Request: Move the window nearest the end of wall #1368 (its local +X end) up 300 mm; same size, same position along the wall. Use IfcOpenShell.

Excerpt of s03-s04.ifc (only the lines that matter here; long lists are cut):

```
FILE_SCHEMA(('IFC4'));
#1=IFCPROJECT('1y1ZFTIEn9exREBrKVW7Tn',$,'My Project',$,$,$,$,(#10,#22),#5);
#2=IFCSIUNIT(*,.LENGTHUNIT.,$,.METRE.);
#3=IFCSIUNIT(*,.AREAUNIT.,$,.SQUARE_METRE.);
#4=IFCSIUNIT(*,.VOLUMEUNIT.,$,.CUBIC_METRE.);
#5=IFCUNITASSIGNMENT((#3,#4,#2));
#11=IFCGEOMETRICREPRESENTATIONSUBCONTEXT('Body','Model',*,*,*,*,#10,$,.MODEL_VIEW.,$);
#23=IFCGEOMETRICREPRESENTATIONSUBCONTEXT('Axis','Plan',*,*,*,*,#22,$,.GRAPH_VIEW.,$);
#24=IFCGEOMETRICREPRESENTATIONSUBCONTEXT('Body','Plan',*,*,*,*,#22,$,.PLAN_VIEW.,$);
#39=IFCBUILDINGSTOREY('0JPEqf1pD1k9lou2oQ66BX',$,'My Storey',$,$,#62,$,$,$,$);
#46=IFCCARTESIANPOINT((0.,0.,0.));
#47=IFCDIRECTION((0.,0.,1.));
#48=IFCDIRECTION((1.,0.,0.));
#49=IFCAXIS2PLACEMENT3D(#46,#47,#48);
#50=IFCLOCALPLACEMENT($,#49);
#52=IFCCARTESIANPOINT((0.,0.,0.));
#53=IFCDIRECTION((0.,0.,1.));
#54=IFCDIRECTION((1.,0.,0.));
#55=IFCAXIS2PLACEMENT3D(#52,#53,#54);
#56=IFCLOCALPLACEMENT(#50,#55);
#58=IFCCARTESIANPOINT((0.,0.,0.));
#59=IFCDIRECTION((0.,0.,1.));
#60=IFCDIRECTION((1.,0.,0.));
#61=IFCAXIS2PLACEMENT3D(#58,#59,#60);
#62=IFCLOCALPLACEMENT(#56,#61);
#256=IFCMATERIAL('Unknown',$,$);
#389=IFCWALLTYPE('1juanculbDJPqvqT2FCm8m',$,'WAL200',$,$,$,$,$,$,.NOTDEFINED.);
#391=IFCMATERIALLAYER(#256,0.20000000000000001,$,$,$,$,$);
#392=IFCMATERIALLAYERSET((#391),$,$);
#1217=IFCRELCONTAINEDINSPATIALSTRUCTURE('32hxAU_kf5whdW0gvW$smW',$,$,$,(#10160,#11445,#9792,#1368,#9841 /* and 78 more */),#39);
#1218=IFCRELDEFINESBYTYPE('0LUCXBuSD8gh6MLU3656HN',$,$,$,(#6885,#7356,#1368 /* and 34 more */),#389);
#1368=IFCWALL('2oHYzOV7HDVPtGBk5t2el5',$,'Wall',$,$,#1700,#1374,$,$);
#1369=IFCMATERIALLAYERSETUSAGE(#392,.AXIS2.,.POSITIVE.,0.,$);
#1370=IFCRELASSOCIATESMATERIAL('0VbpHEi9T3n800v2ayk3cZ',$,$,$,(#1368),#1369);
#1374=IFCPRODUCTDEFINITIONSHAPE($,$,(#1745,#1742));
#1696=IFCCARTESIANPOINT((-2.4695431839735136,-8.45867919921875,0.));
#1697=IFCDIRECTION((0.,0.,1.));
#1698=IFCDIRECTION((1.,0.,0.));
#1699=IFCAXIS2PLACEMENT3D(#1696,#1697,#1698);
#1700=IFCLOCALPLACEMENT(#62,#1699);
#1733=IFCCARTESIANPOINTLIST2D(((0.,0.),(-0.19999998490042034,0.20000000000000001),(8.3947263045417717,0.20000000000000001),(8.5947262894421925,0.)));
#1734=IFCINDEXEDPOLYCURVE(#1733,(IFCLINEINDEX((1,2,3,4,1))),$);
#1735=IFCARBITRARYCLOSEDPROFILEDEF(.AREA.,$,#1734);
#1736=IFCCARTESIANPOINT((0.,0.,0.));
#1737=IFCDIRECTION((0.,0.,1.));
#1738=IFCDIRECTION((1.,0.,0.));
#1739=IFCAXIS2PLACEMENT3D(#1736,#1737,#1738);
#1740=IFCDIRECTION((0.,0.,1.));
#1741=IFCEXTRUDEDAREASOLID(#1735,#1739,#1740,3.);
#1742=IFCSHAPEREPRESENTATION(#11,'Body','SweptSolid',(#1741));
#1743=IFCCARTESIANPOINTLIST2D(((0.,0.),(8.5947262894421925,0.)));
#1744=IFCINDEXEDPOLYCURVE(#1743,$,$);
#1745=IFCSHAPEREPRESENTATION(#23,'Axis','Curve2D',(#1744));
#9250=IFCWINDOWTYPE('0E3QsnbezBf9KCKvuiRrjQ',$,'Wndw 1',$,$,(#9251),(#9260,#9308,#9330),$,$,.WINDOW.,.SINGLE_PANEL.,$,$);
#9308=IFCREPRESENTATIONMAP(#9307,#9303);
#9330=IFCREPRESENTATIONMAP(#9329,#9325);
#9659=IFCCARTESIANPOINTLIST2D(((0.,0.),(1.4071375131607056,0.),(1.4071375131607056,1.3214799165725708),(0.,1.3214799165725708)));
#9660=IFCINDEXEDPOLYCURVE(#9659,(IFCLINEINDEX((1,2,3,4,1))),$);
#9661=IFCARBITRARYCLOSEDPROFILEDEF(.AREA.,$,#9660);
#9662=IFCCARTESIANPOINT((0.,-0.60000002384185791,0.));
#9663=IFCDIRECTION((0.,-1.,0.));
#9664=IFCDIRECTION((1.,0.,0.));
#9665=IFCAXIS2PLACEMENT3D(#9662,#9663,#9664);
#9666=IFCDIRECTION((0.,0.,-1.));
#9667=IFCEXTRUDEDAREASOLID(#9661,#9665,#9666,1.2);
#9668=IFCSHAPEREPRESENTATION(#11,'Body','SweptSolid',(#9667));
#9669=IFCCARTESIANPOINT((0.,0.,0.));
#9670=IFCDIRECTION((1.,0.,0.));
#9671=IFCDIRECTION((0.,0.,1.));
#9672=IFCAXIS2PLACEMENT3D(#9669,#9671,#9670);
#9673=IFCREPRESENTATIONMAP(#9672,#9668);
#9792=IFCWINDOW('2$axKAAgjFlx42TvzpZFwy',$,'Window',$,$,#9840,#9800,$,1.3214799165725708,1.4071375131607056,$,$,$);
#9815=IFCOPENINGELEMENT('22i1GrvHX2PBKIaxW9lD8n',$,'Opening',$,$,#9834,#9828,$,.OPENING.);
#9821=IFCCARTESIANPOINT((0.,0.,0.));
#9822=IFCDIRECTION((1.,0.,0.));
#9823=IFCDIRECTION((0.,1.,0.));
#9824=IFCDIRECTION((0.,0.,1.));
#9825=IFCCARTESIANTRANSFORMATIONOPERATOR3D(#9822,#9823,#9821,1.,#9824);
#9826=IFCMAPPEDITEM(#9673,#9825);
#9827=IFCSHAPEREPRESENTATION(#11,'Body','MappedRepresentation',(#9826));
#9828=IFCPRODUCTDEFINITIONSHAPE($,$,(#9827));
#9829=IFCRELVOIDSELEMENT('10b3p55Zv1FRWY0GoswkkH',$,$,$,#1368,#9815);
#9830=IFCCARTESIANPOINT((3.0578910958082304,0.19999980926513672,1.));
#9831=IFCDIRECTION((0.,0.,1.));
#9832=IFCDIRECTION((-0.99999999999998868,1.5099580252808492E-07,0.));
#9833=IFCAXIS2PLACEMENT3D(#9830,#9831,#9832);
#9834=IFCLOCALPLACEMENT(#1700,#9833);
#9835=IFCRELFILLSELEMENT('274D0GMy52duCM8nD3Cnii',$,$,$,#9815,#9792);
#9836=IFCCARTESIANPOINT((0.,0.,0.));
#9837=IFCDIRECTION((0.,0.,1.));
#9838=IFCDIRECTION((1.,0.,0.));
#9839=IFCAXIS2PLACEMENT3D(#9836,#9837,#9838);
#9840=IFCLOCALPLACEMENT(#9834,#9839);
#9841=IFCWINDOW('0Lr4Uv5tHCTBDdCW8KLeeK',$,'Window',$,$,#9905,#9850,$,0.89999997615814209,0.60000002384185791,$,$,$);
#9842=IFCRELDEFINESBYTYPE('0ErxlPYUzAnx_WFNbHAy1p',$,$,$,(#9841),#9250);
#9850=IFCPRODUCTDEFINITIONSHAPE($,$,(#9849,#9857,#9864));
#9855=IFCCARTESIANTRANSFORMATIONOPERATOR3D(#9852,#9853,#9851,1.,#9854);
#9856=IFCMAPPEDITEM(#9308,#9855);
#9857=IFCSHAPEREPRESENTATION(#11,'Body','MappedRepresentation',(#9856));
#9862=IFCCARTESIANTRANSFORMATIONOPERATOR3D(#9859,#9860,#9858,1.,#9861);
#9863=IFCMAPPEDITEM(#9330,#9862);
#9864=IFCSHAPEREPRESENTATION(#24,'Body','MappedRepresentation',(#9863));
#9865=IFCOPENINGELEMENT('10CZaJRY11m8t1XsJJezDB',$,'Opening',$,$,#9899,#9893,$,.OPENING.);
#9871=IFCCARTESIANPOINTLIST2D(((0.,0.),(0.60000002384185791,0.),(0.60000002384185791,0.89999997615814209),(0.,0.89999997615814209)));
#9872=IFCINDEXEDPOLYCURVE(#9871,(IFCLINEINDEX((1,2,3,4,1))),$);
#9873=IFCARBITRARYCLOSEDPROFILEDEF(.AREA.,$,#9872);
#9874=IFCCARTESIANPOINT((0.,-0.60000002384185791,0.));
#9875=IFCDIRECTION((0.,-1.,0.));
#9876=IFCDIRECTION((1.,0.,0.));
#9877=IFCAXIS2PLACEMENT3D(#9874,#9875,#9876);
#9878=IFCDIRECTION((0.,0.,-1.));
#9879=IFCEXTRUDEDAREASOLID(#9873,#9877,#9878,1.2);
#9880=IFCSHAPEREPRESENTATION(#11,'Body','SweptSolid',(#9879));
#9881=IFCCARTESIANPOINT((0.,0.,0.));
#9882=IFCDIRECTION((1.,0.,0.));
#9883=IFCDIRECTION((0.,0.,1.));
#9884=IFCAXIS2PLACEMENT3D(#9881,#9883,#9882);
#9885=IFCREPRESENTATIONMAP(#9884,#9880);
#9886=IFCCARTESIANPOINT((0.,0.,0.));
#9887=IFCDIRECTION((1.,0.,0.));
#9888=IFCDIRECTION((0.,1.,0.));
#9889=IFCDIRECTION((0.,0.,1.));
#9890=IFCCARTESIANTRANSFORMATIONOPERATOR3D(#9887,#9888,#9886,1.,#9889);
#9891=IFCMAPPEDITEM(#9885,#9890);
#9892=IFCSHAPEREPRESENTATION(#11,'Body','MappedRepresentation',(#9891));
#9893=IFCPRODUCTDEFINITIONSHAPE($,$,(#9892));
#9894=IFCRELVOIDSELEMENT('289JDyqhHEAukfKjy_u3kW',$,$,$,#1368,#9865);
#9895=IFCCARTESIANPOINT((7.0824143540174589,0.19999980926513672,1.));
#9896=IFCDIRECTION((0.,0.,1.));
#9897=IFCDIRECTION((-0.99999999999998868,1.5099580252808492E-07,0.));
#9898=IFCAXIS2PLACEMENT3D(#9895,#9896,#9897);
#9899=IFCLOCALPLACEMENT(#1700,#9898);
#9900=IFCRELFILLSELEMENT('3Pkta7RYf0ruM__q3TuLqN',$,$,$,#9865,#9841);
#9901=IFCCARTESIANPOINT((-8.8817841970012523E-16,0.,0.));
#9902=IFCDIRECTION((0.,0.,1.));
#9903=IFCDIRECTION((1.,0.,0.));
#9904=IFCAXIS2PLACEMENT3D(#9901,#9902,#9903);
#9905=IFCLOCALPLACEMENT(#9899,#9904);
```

```python
import numpy as np
import ifcopenshell
import ifcopenshell.api.geometry
import ifcopenshell.util.placement
import ifcopenshell.util.unit

model = ifcopenshell.open("s03-s04.ifc")
unit_scale = ifcopenshell.util.unit.calculate_unit_scale(model)

window = model.by_guid("0Lr4Uv5tHCTBDdCW8KLeeK")
opening = window.FillsVoids[0].RelatingOpeningElement
dz = 0.3

shift = np.array([0.0, 0.0, dz])
# The window is placed relative to its opening, so it follows when the opening moves.
matrix = ifcopenshell.util.placement.get_local_placement(opening.ObjectPlacement)
matrix[:3, 3] += shift
ifcopenshell.api.geometry.edit_object_placement(
    model, product=opening, matrix=matrix, is_si=False, should_transform_children=True
)

print(f"moved by {dz * unit_scale:+.3f} m")

model.write("s03-s04_updated.ifc")
```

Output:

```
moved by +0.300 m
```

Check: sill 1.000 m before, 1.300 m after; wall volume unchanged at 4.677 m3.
